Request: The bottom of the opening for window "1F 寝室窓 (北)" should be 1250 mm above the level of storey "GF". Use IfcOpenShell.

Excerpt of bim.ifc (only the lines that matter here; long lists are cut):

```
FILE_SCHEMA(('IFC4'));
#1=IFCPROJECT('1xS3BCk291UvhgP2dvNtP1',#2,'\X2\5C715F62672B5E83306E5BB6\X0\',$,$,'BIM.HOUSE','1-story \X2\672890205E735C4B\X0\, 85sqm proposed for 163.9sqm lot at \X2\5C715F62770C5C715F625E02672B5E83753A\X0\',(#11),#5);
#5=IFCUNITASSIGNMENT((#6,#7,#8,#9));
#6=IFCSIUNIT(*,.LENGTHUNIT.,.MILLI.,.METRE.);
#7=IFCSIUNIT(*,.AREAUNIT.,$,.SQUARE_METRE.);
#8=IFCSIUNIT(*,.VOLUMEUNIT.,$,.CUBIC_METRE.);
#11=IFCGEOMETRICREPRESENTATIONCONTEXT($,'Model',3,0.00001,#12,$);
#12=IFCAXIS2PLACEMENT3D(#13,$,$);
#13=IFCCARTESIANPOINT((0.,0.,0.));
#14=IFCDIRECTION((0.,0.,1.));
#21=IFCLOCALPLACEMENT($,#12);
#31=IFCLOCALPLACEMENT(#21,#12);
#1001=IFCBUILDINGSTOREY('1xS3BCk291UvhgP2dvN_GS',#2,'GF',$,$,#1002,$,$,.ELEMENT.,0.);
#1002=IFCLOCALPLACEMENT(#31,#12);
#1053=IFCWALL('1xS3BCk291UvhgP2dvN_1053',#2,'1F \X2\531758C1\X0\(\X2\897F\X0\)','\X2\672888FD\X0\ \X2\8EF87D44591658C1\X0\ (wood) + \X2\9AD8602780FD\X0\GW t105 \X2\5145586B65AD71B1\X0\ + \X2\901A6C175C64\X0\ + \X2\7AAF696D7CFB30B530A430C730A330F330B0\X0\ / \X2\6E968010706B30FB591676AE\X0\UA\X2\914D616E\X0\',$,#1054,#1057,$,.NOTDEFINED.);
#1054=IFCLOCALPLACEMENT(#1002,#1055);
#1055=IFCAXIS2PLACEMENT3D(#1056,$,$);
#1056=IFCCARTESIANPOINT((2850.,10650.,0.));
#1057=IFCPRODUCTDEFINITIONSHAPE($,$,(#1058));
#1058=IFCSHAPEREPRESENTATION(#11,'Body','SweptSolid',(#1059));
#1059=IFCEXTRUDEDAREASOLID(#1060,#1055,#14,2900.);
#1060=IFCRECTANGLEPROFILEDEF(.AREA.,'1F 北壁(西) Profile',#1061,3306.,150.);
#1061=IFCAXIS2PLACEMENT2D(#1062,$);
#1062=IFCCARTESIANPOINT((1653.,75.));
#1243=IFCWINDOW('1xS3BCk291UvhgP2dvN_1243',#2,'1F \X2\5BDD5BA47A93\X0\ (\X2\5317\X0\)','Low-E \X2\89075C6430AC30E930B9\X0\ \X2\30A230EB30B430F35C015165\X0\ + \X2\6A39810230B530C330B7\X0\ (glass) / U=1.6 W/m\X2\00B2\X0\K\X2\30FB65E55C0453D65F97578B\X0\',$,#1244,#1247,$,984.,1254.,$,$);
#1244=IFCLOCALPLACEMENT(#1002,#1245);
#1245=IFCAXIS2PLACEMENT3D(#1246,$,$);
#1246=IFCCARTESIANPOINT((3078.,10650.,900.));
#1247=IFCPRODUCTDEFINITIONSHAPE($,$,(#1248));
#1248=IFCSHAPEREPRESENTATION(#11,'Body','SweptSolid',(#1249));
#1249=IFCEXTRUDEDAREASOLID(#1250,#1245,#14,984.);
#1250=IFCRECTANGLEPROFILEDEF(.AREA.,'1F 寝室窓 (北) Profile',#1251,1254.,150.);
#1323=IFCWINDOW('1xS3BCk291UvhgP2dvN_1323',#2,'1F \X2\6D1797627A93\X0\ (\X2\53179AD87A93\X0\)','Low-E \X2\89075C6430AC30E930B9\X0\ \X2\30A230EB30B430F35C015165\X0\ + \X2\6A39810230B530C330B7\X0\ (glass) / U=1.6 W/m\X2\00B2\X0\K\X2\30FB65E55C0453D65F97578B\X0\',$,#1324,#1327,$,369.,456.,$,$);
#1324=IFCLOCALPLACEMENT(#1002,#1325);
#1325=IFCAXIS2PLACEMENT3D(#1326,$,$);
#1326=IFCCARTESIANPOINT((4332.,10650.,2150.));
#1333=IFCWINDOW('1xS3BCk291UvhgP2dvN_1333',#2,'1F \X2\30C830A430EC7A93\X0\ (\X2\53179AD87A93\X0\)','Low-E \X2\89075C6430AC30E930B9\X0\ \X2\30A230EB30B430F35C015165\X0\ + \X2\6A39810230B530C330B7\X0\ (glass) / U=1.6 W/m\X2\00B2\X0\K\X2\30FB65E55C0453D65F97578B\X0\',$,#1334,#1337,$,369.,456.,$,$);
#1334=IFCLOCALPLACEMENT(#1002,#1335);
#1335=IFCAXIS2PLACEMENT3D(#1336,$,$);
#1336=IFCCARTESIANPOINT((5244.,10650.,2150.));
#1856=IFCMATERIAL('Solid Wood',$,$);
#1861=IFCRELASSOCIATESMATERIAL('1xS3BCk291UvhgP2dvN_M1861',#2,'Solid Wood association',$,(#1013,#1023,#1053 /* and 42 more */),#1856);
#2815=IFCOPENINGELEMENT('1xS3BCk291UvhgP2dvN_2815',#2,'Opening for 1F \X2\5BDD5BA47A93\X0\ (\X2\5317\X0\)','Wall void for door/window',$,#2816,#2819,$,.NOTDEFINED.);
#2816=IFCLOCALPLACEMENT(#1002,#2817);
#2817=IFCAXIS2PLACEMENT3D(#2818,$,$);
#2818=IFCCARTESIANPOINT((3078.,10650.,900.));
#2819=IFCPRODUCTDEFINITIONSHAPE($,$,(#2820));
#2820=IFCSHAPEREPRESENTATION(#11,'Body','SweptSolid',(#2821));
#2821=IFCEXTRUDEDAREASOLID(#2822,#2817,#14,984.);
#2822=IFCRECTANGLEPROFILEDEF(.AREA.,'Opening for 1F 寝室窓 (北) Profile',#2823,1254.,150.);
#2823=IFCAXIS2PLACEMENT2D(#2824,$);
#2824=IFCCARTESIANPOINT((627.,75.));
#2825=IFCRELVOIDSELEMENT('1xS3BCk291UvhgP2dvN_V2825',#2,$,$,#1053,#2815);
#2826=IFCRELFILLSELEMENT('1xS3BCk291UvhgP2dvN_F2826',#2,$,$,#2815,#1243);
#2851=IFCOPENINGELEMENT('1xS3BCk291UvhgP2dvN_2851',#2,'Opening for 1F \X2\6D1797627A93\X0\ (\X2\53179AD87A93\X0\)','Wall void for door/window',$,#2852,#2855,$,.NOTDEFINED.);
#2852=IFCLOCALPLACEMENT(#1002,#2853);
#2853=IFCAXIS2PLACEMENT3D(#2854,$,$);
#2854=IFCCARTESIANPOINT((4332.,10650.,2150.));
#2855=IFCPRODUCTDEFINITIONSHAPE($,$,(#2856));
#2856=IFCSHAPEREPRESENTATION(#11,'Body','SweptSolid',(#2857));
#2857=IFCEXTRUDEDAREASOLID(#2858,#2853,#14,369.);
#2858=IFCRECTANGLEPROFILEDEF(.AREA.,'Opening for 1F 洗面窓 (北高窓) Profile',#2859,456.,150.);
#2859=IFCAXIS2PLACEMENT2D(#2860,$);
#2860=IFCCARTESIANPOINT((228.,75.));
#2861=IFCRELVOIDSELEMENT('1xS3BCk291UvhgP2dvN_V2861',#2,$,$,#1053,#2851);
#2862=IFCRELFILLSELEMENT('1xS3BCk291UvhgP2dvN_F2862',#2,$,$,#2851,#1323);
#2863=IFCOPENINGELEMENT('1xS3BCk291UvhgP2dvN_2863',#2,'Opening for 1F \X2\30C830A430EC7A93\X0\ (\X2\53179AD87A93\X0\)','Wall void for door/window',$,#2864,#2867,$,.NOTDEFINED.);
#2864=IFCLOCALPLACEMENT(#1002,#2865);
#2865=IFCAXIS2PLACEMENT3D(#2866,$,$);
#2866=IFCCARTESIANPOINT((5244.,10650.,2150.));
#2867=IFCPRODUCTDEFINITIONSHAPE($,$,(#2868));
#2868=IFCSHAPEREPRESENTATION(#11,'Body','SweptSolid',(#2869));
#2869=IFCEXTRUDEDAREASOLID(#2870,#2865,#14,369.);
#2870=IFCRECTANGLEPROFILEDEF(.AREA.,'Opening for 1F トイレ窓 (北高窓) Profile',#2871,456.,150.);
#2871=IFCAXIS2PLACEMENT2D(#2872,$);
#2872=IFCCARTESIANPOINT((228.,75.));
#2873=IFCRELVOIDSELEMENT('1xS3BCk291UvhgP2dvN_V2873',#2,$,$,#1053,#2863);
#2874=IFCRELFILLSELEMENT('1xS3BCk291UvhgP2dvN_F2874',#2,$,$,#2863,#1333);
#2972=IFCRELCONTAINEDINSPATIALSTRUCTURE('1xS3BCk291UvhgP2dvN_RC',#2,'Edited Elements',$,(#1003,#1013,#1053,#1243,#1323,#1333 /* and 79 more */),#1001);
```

```python
import numpy as np
import ifcopenshell
import ifcopenshell.api.geometry
import ifcopenshell.geom
import ifcopenshell.util.element
import ifcopenshell.util.placement
import ifcopenshell.util.shape
import ifcopenshell.util.unit

model = ifcopenshell.open("bim.ifc")
unit_scale = ifcopenshell.util.unit.calculate_unit_scale(model)

window = model.by_guid("1xS3BCk291UvhgP2dvN_1243")
opening = window.FillsVoids[0].RelatingOpeningElement
storey = ifcopenshell.util.element.get_container(window, ifc_class="IfcBuildingStorey")
level = ifcopenshell.util.placement.get_local_placement(storey.ObjectPlacement)[2, 3]

# The opening's origin need not be at the sill, so measure its lowest point.
shape = ifcopenshell.geom.create_shape(ifcopenshell.geom.settings(), opening)
bottom = ifcopenshell.util.shape.get_shape_bottom_elevation(shape, shape.geometry) / unit_scale
dz = level + 1.25 / unit_scale - bottom

shift = np.array([0.0, 0.0, dz])
# The window is not placed relative to its opening, so move both.
for product in (opening, window):
    matrix = ifcopenshell.util.placement.get_local_placement(product.ObjectPlacement)
    matrix[:3, 3] += shift
    ifcopenshell.api.geometry.edit_object_placement(model, product=product, matrix=matrix, is_si=False)

print(f"moved by {dz * unit_scale:+.3f} m")

model.write("bim-out.ifc")
```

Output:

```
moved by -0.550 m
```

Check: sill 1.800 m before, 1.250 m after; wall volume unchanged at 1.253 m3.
